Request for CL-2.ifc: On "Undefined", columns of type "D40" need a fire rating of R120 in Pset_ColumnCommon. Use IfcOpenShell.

First a look at what the model holds.

```python
import ifcopenshell
import ifcopenshell.util.element

model = ifcopenshell.open("CL-2.ifc")
print(model.schema)
storey = next(s for s in model.by_type("IfcBuildingStorey") if s.Name == "Undefined")
columns = [e for e in ifcopenshell.util.element.get_decomposition(storey) if e.is_a("IfcColumn")]
seen = {}
for e in columns:
    element_type = ifcopenshell.util.element.get_type(e)
    key = (element_type.Name if element_type != e and element_type else None, ifcopenshell.util.element.get_pset(e, "Pset_ColumnCommon", "FireRating"))
    seen[key] = seen.get(key, 0) + 1
for (name, value), count in sorted(seen.items(), key=str):
    print(count, "x", name, "|", value)
```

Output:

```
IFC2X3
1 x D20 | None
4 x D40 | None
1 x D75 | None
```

```python
import ifcopenshell
import ifcopenshell.api.pset
import ifcopenshell.util.element

model = ifcopenshell.open("CL-2.ifc")

storey = next(s for s in model.by_type("IfcBuildingStorey") if s.Name == "Undefined")
columns = [e for e in ifcopenshell.util.element.get_decomposition(storey) if e.is_a("IfcColumn")]

count = 0
for e in columns:
    element_type = ifcopenshell.util.element.get_type(e)
    if element_type in (None, e) or element_type.Name != "D40":
        continue
    found = ifcopenshell.util.element.get_pset(e, "Pset_ColumnCommon", should_inherit=False)
    if found:
        pset = model.by_id(found["id"])
        if len(ifcopenshell.util.element.get_elements_by_pset(pset)) > 1:
            pset = ifcopenshell.api.pset.unshare_pset(model, products=[e], pset=pset)[0]
    else:
        pset = ifcopenshell.api.pset.add_pset(model, product=e, name="Pset_ColumnCommon")
    ifcopenshell.api.pset.edit_pset(model, pset=pset, properties={"FireRating": "R120"})
    count += 1

print(count, "columns updated")

model.write("CL-2_v2.ifc")
```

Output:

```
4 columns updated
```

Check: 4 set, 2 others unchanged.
